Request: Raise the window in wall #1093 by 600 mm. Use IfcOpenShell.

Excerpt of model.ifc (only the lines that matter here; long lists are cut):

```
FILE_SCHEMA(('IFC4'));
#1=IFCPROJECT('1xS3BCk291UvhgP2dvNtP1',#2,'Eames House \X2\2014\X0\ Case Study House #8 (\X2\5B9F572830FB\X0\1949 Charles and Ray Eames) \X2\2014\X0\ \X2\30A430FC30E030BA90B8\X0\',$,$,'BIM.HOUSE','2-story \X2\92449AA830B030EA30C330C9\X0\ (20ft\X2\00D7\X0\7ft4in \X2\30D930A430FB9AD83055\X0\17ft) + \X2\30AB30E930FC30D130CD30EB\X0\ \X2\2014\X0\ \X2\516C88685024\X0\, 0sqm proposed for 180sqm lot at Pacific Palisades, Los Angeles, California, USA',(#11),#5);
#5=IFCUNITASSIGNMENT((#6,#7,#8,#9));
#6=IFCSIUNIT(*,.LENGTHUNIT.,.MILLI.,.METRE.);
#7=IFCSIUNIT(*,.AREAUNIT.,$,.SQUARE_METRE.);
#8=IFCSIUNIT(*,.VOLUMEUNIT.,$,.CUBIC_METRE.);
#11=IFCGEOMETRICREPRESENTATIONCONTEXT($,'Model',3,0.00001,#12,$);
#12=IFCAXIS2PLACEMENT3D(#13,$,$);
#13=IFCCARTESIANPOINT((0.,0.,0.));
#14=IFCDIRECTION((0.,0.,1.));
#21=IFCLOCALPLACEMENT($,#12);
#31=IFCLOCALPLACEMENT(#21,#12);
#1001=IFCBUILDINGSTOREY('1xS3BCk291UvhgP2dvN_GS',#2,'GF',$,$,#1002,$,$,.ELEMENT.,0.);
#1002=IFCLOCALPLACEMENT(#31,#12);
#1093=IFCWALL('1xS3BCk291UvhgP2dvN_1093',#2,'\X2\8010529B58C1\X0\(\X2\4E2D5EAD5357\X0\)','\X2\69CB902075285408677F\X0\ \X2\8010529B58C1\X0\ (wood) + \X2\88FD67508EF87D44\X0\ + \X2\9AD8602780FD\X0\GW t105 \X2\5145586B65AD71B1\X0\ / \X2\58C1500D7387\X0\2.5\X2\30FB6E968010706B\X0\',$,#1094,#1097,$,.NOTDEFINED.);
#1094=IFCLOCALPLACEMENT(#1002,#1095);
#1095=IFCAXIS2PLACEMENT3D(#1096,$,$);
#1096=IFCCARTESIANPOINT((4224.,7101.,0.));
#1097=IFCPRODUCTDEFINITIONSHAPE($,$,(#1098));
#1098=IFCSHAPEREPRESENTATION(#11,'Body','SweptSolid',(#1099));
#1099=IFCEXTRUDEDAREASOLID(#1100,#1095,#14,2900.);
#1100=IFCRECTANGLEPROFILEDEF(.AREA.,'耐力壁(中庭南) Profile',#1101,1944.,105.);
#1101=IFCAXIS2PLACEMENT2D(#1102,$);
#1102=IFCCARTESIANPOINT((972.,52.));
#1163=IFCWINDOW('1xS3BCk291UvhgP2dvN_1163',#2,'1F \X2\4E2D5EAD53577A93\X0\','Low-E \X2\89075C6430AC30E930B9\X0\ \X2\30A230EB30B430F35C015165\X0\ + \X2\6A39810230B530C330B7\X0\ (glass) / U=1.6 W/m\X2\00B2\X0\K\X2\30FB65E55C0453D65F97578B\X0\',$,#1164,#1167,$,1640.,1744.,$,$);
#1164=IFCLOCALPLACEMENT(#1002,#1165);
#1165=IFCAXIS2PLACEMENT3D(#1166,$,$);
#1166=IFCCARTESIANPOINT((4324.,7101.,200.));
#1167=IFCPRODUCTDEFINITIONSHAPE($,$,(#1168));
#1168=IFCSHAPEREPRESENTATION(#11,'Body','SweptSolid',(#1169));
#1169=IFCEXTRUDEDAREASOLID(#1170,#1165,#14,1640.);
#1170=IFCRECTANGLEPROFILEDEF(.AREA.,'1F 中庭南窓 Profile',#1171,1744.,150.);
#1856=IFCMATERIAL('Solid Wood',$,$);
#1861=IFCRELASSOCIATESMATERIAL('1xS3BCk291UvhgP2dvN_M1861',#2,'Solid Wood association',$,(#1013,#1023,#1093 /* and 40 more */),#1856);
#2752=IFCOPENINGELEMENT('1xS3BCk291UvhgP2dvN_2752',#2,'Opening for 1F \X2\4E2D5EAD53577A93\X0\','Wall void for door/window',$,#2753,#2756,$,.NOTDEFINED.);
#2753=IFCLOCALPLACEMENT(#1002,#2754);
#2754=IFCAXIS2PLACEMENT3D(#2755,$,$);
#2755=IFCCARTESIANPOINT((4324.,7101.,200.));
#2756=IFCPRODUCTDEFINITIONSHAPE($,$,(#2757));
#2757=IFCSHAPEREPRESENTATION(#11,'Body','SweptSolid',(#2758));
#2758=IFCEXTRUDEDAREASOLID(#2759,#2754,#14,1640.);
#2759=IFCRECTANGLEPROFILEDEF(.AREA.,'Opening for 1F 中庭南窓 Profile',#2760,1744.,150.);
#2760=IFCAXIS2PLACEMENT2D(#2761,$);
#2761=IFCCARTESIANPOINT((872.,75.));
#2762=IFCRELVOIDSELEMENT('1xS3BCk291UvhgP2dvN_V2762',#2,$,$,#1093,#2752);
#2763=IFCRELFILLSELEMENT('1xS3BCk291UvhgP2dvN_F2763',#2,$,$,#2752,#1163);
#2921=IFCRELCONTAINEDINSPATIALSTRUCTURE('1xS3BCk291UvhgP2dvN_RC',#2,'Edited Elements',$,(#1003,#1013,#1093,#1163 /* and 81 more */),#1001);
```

```python
import numpy as np
import ifcopenshell
import ifcopenshell.api.geometry
import ifcopenshell.util.placement
import ifcopenshell.util.unit

model = ifcopenshell.open("model.ifc")
unit_scale = ifcopenshell.util.unit.calculate_unit_scale(model)

window = model.by_id(1163)
opening = window.FillsVoids[0].RelatingOpeningElement
dz = 600.0

shift = np.array([0.0, 0.0, dz])
# The window is not placed relative to its opening, so move both.
for product in (opening, window):
    matrix = ifcopenshell.util.placement.get_local_placement(product.ObjectPlacement)
    matrix[:3, 3] += shift
    ifcopenshell.api.geometry.edit_object_placement(model, product=product, matrix=matrix, is_si=False)

print(f"moved by {dz * unit_scale:+.3f} m")

model.write("model_updated.ifc")
```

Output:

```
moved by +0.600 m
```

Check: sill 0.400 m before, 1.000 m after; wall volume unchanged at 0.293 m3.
